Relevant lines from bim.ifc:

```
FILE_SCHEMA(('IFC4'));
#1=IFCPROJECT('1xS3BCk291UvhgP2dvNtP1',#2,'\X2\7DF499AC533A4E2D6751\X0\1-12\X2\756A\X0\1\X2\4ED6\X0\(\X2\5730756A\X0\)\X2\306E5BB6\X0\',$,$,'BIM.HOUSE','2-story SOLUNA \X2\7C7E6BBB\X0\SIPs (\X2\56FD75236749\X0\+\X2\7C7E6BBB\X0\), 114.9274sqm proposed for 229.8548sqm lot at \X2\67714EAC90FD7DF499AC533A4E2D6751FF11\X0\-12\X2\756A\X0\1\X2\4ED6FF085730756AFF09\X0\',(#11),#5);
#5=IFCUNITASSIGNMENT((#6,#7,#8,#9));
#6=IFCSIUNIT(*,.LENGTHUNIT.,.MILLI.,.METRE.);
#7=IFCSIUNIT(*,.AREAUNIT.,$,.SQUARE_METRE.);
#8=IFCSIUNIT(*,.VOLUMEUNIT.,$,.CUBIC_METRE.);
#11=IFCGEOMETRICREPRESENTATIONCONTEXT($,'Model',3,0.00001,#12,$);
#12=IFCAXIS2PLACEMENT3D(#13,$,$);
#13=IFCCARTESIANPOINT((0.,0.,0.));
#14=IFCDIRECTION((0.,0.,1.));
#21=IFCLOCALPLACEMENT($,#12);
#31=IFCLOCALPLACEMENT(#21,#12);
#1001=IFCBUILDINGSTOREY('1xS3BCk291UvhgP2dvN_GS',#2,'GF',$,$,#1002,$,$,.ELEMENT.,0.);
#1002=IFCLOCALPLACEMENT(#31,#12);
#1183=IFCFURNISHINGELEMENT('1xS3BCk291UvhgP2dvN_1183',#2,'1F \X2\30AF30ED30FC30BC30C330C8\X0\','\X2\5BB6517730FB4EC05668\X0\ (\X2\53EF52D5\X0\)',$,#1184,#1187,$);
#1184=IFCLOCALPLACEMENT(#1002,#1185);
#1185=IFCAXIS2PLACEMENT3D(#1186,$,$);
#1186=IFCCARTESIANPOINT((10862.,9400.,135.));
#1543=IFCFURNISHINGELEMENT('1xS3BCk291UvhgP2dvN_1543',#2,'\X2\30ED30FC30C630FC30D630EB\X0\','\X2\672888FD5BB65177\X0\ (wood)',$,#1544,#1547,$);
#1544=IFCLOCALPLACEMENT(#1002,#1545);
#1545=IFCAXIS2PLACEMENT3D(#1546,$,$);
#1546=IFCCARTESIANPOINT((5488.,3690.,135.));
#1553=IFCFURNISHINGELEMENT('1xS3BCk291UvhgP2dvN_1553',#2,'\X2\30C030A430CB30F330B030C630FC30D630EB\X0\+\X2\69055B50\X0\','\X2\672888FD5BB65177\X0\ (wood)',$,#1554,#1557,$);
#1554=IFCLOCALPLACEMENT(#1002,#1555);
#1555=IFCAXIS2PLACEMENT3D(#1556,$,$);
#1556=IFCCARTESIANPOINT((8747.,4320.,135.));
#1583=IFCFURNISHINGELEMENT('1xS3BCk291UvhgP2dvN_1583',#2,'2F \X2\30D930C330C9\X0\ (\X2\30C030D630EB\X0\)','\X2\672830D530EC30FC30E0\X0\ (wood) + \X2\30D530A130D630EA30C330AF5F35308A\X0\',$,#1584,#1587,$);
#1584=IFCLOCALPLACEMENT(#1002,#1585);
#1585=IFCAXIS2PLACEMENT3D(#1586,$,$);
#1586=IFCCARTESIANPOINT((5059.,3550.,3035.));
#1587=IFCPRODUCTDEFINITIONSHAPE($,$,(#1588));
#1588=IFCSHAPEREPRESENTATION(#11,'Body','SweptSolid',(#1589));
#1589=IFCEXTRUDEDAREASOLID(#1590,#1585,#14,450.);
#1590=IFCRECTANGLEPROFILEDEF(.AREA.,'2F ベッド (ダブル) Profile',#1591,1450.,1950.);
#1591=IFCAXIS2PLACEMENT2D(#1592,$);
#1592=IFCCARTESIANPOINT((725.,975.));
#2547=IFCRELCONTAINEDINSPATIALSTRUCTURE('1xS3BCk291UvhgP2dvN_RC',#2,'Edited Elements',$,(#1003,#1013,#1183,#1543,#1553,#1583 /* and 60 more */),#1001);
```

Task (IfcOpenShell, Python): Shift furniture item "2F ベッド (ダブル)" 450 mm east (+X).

```python
import ifcopenshell
import ifcopenshell.api.geometry
import ifcopenshell.util.placement
import ifcopenshell.util.unit

model = ifcopenshell.open("bim.ifc")
unit_scale = ifcopenshell.util.unit.calculate_unit_scale(model)

item = model.by_guid("1xS3BCk291UvhgP2dvN_1583")
matrix = ifcopenshell.util.placement.get_local_placement(item.ObjectPlacement)
matrix[0, 3] += 0.45 / unit_scale
ifcopenshell.api.geometry.edit_object_placement(model, product=item, matrix=matrix, is_si=False)

print(ifcopenshell.util.placement.get_local_placement(item.ObjectPlacement).round(3) + 0.0)

model.write("bim_v2.ifc")
```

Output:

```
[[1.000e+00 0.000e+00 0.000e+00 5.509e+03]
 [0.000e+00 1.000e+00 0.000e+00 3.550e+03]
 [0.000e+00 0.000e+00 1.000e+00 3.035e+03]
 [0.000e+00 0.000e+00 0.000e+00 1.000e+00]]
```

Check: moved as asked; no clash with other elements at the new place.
